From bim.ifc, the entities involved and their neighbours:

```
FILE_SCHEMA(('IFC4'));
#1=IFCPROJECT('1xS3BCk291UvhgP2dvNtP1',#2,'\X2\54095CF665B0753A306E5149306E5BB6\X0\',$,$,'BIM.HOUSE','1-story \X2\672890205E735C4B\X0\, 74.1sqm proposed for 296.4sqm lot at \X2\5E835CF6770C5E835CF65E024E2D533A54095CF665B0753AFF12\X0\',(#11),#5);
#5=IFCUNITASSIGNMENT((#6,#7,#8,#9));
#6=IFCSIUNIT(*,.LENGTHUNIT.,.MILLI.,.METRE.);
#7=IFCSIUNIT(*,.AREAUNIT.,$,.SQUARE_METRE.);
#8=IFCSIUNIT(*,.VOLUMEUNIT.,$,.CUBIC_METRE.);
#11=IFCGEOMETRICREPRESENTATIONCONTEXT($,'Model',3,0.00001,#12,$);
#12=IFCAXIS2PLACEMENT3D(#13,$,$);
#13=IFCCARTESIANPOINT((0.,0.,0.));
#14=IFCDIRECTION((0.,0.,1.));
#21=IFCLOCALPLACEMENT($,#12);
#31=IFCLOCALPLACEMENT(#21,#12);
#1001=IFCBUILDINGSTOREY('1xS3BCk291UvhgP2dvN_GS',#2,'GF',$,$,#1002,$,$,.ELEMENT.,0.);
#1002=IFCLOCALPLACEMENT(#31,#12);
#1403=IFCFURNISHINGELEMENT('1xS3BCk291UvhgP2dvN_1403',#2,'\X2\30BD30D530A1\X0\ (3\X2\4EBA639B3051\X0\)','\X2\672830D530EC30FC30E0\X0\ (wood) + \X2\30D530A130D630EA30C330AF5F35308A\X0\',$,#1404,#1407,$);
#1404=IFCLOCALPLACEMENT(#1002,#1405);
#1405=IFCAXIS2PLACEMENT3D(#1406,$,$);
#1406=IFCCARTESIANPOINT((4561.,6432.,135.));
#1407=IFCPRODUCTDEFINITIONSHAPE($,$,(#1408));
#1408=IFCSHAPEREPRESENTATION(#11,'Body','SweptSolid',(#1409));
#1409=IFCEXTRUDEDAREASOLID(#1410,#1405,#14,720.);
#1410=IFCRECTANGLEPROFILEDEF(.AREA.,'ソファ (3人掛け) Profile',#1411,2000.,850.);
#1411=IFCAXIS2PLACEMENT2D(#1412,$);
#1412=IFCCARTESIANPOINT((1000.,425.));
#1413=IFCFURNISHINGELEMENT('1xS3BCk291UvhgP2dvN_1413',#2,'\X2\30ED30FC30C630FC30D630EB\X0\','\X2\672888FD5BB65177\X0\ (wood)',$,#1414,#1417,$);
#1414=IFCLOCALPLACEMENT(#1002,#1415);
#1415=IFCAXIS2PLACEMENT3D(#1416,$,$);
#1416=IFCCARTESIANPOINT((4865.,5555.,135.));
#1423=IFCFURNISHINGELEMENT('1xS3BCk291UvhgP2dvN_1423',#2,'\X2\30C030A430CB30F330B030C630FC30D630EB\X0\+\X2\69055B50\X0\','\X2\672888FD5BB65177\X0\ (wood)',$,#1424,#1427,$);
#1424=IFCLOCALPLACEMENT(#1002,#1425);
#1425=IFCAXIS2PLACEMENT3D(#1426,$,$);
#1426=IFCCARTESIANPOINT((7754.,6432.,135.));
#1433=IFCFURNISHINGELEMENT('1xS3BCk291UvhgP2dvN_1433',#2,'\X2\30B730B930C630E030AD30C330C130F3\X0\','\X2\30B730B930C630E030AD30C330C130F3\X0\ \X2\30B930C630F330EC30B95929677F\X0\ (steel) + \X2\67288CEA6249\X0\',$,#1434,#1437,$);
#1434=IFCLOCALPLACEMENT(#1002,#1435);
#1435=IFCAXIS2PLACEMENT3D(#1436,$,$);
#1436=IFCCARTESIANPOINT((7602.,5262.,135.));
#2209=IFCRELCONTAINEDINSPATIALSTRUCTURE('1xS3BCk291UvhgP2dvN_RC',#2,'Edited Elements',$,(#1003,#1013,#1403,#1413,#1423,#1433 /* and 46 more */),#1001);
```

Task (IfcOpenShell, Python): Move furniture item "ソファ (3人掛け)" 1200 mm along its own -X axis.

```python
import ifcopenshell
import ifcopenshell.api.geometry
import ifcopenshell.util.placement
import ifcopenshell.util.unit

model = ifcopenshell.open("bim.ifc")
unit_scale = ifcopenshell.util.unit.calculate_unit_scale(model)

item = model.by_guid("1xS3BCk291UvhgP2dvN_1403")
matrix = ifcopenshell.util.placement.get_local_placement(item.ObjectPlacement)
matrix[:3, 3] -= matrix[:3, 0] * 1.2 / unit_scale
ifcopenshell.api.geometry.edit_object_placement(model, product=item, matrix=matrix, is_si=False)

print(ifcopenshell.util.placement.get_local_placement(item.ObjectPlacement).round(3) + 0.0)

model.write("bim_edited.ifc")
```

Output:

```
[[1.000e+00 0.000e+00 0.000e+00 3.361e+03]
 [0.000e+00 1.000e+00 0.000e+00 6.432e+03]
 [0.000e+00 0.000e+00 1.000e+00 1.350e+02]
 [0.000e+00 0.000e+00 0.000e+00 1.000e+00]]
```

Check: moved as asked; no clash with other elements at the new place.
